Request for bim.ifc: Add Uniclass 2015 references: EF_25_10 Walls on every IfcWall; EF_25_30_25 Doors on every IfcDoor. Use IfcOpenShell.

First a look at what the model holds.

```python
import ifcopenshell

model = ifcopenshell.open("bim.ifc")
print(model.schema)
print("classifications:", [c.Name for c in model.by_type("IfcClassification")])
for ifc_class in ("IfcDoor", "IfcRoof", "IfcStair", "IfcWall", "IfcWindow"):
    print(ifc_class, len(model.by_type(ifc_class)))
```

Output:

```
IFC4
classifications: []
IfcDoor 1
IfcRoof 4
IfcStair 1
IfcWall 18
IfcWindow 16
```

```python
import ifcopenshell
import ifcopenshell.api.classification

model = ifcopenshell.open("bim.ifc")

system = ifcopenshell.api.classification.add_classification(model, classification="Uniclass 2015")

codes = {
    "IfcWall": ("EF_25_10", "Walls"),
    "IfcDoor": ("EF_25_30_25", "Doors"),
}
for ifc_class, (code, name) in codes.items():
    products = model.by_type(ifc_class)
    ifcopenshell.api.classification.add_reference(
        model, products=products, classification=system, identification=code, name=name
    )
    print(code, len(products))

model.write("bim_edited.ifc")
```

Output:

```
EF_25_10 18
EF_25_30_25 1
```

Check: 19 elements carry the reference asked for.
